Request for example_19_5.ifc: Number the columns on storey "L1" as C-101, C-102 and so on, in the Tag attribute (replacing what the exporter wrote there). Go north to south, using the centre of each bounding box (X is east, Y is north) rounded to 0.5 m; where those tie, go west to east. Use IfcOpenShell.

First a look at what the model holds.

```python
import ifcopenshell
import ifcopenshell.util.element
import ifcopenshell.util.placement

model = ifcopenshell.open("example_19_5.ifc")
print(model.schema)
storey = next(s for s in model.by_type("IfcBuildingStorey") if s.Name == "L1")
columns = [e for e in ifcopenshell.util.element.get_decomposition(storey) if e.is_a("IfcColumn")]
for e in sorted(columns, key=lambda e: e.id()):
    origin = ifcopenshell.util.placement.get_local_placement(e.ObjectPlacement)[:3, 3]
    print(e.id(), e.Tag, e.Name, origin.round(2) + 0.0, sep=" | ")
```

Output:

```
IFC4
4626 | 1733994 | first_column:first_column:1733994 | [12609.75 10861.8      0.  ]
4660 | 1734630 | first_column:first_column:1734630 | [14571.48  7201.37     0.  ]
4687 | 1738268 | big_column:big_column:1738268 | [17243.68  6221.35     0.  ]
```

```python
import ifcopenshell
import ifcopenshell.geom
import ifcopenshell.util.element
import ifcopenshell.util.shape

model = ifcopenshell.open("example_19_5.ifc")
settings = ifcopenshell.geom.settings()
settings.set("use-world-coords", True)


def centre(element):
    shape = ifcopenshell.geom.create_shape(settings, element)
    return ifcopenshell.util.shape.get_bbox_centroid(shape.geometry)


storey = next(s for s in model.by_type("IfcBuildingStorey") if s.Name == "L1")
columns = [e for e in ifcopenshell.util.element.get_decomposition(storey) if e.is_a("IfcColumn")]

# Insertion points can sit at a corner or the storey origin, so sort by the geometry (in metres).
centres = {e: centre(e) for e in columns}
columns.sort(key=lambda e: (-round(centres[e][1] / 0.5), centres[e][0]))

for i, e in enumerate(columns, start=1):
    number = f"C-1{i:02d}"
    e.Tag = number
    print(e.id(), number)

model.write("example_19_5_edited.ifc")
```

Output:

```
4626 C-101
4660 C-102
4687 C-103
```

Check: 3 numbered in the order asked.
